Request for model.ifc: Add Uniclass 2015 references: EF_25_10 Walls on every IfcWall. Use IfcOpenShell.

First a look at what the model holds.

```python
import ifcopenshell

model = ifcopenshell.open("model.ifc")
print(model.schema)
print("classifications:", [c.Name for c in model.by_type("IfcClassification")])
for ifc_class in ("IfcDoor", "IfcRoof", "IfcStair", "IfcWall", "IfcWindow"):
    print(ifc_class, len(model.by_type(ifc_class)))
```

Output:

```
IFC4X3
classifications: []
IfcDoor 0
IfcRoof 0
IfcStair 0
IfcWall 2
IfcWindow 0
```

```python
import ifcopenshell
import ifcopenshell.api.classification

model = ifcopenshell.open("model.ifc")

system = ifcopenshell.api.classification.add_classification(model, classification="Uniclass 2015")

codes = {
    "IfcWall": ("EF_25_10", "Walls"),
}
for ifc_class, (code, name) in codes.items():
    products = model.by_type(ifc_class)
    ifcopenshell.api.classification.add_reference(
        model, products=products, classification=system, identification=code, name=name
    )
    print(code, len(products))

model.write("model-out.ifc")
```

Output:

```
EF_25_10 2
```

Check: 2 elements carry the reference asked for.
